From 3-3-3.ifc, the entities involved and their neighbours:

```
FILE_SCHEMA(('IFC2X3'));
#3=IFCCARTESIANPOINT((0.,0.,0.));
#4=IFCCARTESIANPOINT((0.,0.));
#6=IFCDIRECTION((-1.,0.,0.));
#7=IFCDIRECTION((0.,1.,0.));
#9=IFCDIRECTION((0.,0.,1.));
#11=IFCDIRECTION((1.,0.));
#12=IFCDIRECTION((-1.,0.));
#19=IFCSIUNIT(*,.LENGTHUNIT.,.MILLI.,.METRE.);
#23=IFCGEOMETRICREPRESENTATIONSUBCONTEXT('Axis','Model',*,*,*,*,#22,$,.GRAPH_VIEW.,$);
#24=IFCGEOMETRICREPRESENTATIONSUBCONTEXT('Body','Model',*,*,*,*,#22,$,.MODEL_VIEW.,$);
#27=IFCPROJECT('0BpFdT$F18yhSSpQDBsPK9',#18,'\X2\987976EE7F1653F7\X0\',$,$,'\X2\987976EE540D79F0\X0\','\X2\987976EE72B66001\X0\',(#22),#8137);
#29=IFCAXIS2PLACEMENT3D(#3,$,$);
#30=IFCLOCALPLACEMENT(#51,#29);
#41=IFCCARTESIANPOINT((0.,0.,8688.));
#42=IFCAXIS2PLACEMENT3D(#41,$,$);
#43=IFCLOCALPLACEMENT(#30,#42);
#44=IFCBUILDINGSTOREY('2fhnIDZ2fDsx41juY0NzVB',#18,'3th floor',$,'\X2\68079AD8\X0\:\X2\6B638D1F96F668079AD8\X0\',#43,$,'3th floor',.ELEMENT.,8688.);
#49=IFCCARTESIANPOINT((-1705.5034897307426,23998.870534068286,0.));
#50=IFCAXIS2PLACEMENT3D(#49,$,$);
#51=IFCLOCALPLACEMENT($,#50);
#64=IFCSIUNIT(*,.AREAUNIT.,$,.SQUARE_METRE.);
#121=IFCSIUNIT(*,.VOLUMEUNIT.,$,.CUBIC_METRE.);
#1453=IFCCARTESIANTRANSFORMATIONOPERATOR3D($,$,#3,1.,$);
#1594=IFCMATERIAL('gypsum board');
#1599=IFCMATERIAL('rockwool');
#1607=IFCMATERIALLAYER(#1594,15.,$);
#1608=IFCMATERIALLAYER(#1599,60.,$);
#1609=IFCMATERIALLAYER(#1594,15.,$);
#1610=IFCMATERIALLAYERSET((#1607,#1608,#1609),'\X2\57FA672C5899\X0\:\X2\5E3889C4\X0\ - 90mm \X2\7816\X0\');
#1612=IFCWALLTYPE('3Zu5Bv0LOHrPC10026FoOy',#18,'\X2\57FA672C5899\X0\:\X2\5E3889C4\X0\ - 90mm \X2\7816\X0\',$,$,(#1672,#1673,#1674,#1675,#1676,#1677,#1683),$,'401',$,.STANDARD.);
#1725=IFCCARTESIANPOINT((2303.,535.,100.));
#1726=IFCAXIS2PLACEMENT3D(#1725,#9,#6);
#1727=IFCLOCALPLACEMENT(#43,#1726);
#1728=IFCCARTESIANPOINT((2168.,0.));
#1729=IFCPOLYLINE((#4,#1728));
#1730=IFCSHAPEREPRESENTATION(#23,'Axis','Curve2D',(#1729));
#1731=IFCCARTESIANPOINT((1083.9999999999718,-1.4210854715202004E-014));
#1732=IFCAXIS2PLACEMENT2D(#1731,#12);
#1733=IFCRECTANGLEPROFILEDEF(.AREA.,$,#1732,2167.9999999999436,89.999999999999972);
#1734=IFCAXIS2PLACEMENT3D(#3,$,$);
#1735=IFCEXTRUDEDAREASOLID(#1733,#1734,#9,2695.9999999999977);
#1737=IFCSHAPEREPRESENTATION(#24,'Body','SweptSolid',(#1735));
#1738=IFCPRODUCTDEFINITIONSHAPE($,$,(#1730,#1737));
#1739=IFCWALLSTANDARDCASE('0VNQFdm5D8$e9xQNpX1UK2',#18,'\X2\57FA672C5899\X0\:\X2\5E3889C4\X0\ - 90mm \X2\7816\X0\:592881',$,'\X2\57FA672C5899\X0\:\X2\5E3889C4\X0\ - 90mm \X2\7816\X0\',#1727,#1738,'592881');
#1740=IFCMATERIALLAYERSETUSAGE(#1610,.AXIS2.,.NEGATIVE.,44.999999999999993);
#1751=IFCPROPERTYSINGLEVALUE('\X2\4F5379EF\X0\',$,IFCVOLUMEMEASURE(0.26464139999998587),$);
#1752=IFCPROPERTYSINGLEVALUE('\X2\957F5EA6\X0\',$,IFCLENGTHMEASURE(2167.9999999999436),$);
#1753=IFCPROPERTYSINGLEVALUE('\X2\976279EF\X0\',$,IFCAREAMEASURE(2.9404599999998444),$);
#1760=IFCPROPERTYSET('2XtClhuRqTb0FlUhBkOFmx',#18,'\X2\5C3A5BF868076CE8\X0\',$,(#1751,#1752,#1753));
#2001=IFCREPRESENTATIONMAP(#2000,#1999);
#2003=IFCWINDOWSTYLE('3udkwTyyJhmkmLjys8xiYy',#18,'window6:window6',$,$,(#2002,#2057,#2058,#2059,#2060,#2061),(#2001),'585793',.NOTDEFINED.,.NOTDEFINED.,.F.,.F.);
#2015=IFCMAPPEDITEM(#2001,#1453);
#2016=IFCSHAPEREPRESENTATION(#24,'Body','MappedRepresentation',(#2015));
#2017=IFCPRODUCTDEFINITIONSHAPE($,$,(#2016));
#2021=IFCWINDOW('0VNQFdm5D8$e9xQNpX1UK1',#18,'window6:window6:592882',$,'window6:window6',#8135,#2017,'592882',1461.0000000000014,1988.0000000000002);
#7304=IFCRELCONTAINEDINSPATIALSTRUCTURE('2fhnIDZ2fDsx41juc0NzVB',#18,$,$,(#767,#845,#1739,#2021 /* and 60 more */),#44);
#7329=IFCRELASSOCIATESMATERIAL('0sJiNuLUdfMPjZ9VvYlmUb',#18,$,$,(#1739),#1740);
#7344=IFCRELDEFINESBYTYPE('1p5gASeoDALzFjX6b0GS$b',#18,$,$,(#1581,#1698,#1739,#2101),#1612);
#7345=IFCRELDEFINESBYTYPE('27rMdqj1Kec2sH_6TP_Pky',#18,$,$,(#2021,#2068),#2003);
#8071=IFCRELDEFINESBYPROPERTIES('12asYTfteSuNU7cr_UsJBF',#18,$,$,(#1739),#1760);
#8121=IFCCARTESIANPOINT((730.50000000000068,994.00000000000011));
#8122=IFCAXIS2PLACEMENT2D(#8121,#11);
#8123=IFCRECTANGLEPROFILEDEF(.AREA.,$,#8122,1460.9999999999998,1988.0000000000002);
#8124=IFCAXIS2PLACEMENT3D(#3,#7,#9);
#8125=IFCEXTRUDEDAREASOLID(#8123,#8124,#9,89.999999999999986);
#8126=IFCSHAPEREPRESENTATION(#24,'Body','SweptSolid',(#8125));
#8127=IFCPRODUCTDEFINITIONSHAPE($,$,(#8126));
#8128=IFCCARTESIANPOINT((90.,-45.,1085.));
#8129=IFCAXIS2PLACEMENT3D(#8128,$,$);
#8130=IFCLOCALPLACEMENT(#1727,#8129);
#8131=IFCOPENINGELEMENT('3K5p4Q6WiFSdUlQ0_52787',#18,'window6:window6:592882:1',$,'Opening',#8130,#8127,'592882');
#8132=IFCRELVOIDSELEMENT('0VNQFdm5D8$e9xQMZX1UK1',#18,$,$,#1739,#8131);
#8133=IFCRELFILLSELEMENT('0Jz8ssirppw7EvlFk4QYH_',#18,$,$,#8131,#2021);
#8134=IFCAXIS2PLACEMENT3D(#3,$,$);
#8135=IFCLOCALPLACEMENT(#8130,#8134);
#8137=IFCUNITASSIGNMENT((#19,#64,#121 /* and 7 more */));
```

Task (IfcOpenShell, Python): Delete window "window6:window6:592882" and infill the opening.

```python
import ifcopenshell
import ifcopenshell.api.feature
import ifcopenshell.api.pset
import ifcopenshell.api.root
import ifcopenshell.geom
import ifcopenshell.util.element
import ifcopenshell.util.shape
import ifcopenshell.util.unit

model = ifcopenshell.open("3-3-3.ifc")
area_scale = ifcopenshell.util.unit.calculate_unit_scale(model, "AREAUNIT")
volume_scale = ifcopenshell.util.unit.calculate_unit_scale(model, "VOLUMEUNIT")
settings = ifcopenshell.geom.settings()


def volume(element):
    """Net volume in cubic metres, openings subtracted."""
    shape = ifcopenshell.geom.create_shape(settings, element)
    return ifcopenshell.util.shape.get_volume(shape.geometry)


window = model.by_guid("0VNQFdm5D8$e9xQNpX1UK1")
opening = window.FillsVoids[0].RelatingOpeningElement
wall = opening.VoidsElements[0].RelatingBuildingElement
before = volume(wall)

ifcopenshell.api.root.remove_product(model, product=window)
ifcopenshell.api.feature.remove_feature(model, feature=opening)

after = volume(wall)
thickness = 0.09  # wall thickness in metres

# Update the wall's stored quantities.
pset = model.by_id(ifcopenshell.util.element.get_pset(wall, "尺寸标注", should_inherit=False)["id"])
ifcopenshell.api.pset.edit_pset(model, pset=pset, properties={
    "体积": model.create_entity("IfcVolumeMeasure", after / volume_scale),
    "面积": model.create_entity("IfcAreaMeasure", after / thickness / area_scale),
})

print(f"wall volume {before:.3f} -> {after:.3f} m3")

model.write("3-3-3_rev.ifc")
```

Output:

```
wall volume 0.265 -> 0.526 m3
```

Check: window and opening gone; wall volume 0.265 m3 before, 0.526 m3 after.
